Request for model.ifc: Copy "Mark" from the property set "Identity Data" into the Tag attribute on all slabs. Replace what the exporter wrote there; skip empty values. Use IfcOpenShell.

First a look at what the model holds.

```python
import ifcopenshell
import ifcopenshell.util.element

model = ifcopenshell.open("model.ifc")
print(model.schema)
slabs = model.by_type("IfcSlab")
print(len(slabs), "slabs")
for e in slabs[:8]:
    source = ifcopenshell.util.element.get_pset(e, "Identity Data", "Mark")
    target = e.Tag
    print(e.id(), repr(source), repr(target), sep=" | ")
```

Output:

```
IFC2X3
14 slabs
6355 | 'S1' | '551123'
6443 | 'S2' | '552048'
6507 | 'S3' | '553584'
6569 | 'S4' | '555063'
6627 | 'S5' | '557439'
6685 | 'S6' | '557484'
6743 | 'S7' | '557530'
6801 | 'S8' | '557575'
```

```python
import ifcopenshell
import ifcopenshell.util.element

model = ifcopenshell.open("model.ifc")

count = 0
for e in model.by_type("IfcSlab"):
    value = ifcopenshell.util.element.get_pset(e, "Identity Data", "Mark")
    current = e.Tag
    if not value or not value.strip() or current == value:
        continue
    e.Tag = value
    count += 1

print(count, "slabs updated")

model.write("model_updated.ifc")
```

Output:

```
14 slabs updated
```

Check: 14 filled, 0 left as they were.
